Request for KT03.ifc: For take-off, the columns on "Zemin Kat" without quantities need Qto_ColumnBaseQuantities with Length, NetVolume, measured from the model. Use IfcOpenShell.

First a look at what the model holds.

```python
import ifcopenshell
import ifcopenshell.util.element
import ifcopenshell.util.unit

model = ifcopenshell.open("KT03.ifc")
print(model.schema)
for unit_type in ("LENGTHUNIT", "AREAUNIT", "VOLUMEUNIT"):
    print(unit_type, ifcopenshell.util.unit.calculate_unit_scale(model, unit_type))
storey = next(s for s in model.by_type("IfcBuildingStorey") if s.Name == "Zemin Kat")
columns = [e for e in ifcopenshell.util.element.get_decomposition(storey) if e.is_a("IfcColumn")]
for e in sorted(columns, key=lambda e: e.id()):
    print(e.id(), e.is_a(), e.Name, list(ifcopenshell.util.element.get_psets(e, qtos_only=True)), sep=" | ")
```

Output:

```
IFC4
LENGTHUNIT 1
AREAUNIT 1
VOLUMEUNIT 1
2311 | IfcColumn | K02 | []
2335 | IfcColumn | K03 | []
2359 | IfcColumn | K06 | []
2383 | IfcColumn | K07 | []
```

```python
import ifcopenshell
import ifcopenshell.api.pset
import ifcopenshell.geom
import ifcopenshell.util.element
import ifcopenshell.util.shape
import ifcopenshell.util.unit

model = ifcopenshell.open("KT03.ifc")
unit_scale = ifcopenshell.util.unit.calculate_unit_scale(model)
volume_scale = ifcopenshell.util.unit.calculate_unit_scale(model, "VOLUMEUNIT")
settings = ifcopenshell.geom.settings()

storey = next(s for s in model.by_type("IfcBuildingStorey") if s.Name == "Zemin Kat")
columns = [e for e in ifcopenshell.util.element.get_decomposition(storey) if e.is_a("IfcColumn")]

for e in sorted(columns, key=lambda e: e.id()):
    if ifcopenshell.util.element.get_psets(e, qtos_only=True, should_inherit=False):
        continue
    # Geometry comes back in metres, in the element's own axes.
    shape = ifcopenshell.geom.create_shape(settings, e)
    values = {
        "Length": ifcopenshell.util.shape.get_z(shape.geometry) / unit_scale,
        "NetVolume": ifcopenshell.util.shape.get_volume(shape.geometry) / volume_scale,
    }
    qto = ifcopenshell.api.pset.add_qto(model, product=e, name="Qto_ColumnBaseQuantities")
    ifcopenshell.api.pset.edit_qto(model, qto=qto, properties=values)
    print(e.id(), {k: round(v, 3) for k, v in values.items()})

model.write("KT03_edited.ifc")
```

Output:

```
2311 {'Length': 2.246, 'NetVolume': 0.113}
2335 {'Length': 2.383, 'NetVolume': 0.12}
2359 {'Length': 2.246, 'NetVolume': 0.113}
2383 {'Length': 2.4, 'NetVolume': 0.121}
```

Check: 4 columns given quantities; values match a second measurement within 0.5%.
